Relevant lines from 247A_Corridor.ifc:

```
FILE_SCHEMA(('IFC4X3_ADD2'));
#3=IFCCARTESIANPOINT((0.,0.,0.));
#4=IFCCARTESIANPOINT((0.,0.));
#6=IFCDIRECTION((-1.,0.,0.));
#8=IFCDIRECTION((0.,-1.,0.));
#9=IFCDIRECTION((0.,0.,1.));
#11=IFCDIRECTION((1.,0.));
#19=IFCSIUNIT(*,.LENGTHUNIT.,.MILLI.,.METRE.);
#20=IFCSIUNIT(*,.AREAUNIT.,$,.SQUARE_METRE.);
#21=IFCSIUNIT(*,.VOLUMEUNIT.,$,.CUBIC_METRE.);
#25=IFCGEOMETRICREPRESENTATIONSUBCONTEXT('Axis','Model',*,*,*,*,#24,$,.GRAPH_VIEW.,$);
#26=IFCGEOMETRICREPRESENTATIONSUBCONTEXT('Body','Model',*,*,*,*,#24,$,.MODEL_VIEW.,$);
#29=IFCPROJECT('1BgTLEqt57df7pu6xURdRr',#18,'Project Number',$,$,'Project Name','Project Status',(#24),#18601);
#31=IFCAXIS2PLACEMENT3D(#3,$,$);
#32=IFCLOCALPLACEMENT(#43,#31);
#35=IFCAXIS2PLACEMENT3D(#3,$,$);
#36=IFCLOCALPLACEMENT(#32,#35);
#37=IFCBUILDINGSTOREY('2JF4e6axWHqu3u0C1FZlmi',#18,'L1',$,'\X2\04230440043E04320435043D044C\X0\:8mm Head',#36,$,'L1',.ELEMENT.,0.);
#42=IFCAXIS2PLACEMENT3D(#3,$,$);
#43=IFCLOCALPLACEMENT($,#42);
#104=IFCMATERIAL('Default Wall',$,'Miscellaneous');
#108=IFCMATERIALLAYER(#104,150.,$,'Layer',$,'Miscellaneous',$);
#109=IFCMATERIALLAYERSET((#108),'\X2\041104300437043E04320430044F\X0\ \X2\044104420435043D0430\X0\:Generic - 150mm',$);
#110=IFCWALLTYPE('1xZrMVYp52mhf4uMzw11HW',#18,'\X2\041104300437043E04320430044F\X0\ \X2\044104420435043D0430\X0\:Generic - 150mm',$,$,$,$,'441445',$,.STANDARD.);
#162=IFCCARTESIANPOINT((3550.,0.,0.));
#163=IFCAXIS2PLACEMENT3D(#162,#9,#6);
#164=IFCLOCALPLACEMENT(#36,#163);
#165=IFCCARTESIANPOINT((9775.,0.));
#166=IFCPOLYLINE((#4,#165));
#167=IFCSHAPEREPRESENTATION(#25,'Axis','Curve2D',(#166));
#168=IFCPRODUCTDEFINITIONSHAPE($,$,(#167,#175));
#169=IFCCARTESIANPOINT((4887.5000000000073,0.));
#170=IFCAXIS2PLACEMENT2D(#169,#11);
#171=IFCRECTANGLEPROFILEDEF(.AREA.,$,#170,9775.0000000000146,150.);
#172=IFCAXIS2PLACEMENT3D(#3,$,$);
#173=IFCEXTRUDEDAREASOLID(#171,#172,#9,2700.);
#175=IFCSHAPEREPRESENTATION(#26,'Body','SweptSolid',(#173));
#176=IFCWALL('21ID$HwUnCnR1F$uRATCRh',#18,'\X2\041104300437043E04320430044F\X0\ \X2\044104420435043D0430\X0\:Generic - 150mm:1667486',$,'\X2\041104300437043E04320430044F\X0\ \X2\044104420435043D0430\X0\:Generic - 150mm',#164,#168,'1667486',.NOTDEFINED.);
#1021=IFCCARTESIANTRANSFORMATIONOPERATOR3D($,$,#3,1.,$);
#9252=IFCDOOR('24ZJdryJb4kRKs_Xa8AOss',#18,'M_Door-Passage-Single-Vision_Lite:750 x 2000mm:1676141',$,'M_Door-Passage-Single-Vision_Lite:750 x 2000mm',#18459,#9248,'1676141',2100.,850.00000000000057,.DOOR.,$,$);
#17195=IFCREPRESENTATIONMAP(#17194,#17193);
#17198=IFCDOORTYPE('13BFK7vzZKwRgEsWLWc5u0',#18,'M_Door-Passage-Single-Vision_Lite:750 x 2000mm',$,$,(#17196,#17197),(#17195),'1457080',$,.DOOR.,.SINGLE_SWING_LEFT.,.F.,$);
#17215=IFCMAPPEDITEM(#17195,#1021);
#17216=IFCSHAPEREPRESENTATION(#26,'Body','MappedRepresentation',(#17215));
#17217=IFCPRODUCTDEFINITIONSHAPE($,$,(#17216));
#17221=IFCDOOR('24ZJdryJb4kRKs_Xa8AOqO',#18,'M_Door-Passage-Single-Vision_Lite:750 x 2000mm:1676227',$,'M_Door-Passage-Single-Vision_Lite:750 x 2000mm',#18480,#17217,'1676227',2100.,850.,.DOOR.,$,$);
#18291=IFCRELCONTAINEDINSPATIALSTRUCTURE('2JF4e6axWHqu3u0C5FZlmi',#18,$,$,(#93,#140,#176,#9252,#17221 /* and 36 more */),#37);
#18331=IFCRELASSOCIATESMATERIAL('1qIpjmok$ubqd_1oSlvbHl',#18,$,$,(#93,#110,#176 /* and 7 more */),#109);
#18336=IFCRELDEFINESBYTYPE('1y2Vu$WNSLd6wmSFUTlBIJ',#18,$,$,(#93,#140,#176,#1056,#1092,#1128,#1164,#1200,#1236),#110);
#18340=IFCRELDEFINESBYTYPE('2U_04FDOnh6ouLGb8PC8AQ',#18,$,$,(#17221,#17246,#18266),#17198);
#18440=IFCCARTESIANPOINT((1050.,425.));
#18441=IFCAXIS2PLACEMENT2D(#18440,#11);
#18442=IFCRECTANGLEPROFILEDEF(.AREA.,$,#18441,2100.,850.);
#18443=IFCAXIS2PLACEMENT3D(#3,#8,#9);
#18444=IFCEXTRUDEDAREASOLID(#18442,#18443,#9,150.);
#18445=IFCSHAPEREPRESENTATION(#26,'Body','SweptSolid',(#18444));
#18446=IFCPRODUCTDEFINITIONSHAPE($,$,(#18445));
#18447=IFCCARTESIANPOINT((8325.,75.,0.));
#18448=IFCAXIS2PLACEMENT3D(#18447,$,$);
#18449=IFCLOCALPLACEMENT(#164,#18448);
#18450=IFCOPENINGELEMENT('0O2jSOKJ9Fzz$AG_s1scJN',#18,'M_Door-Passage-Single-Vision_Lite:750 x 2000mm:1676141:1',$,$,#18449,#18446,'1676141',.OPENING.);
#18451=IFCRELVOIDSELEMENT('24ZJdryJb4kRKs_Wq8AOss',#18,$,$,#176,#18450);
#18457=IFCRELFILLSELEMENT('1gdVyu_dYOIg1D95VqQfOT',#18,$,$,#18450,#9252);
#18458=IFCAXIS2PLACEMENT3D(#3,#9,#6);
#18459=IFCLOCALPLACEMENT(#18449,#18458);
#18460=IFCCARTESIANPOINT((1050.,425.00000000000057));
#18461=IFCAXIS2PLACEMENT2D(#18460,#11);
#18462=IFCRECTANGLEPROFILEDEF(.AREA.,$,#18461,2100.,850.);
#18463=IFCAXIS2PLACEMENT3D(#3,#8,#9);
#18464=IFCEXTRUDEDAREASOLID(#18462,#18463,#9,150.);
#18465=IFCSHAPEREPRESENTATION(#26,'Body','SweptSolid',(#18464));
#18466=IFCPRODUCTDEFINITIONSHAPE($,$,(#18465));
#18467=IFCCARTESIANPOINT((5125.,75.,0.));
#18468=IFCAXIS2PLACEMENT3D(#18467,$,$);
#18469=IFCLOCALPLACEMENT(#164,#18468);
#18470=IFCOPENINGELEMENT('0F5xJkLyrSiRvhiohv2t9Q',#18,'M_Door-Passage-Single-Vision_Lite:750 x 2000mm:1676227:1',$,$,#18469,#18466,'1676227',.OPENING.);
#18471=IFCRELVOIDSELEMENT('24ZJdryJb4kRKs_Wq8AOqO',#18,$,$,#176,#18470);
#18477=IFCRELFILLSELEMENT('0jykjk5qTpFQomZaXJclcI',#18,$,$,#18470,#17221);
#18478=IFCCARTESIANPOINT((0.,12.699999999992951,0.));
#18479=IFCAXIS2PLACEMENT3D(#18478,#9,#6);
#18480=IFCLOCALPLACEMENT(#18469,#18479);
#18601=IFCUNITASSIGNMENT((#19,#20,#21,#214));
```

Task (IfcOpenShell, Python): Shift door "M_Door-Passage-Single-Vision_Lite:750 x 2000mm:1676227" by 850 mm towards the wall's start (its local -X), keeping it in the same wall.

```python
import ifcopenshell
import ifcopenshell.api.geometry
import ifcopenshell.util.placement
import ifcopenshell.util.unit

model = ifcopenshell.open("247A_Corridor.ifc")
unit_scale = ifcopenshell.util.unit.calculate_unit_scale(model)

door = model.by_guid("24ZJdryJb4kRKs_Xa8AOqO")
opening = door.FillsVoids[0].RelatingOpeningElement
wall = opening.VoidsElements[0].RelatingBuildingElement

wall_matrix = ifcopenshell.util.placement.get_local_placement(wall.ObjectPlacement)
shift = wall_matrix[:3, 0] * -0.85 / unit_scale
before = ifcopenshell.util.placement.get_local_placement(door.ObjectPlacement)[:3, 3].copy()

# The door is placed relative to its opening, so it follows when the opening moves.
matrix = ifcopenshell.util.placement.get_local_placement(opening.ObjectPlacement)
matrix[:3, 3] += shift
ifcopenshell.api.geometry.edit_object_placement(
    model, product=opening, matrix=matrix, is_si=False, should_transform_children=True
)

after = ifcopenshell.util.placement.get_local_placement(door.ObjectPlacement)[:3, 3]
print("door moved by", (after - before).round(3) + 0.0)

model.write("247A_Corridor_rev.ifc")
```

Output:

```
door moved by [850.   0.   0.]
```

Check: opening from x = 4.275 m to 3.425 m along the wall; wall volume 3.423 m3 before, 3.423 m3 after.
